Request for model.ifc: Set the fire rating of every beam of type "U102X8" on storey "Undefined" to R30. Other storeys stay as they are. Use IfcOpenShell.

First a look at what the model holds.

```python
import ifcopenshell
import ifcopenshell.util.element

model = ifcopenshell.open("model.ifc")
print(model.schema)
storey = next(s for s in model.by_type("IfcBuildingStorey") if s.Name == "Undefined")
beams = [e for e in ifcopenshell.util.element.get_decomposition(storey) if e.is_a("IfcBeam")]
seen = {}
for e in beams:
    element_type = ifcopenshell.util.element.get_type(e)
    key = (element_type.Name if element_type != e and element_type else None, ifcopenshell.util.element.get_pset(e, "Pset_BeamCommon", "FireRating"))
    seen[key] = seen.get(key, 0) + 1
for (name, value), count in sorted(seen.items(), key=str):
    print(count, "x", name, "|", value)
```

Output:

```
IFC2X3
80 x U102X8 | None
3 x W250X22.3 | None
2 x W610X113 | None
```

```python
import ifcopenshell
import ifcopenshell.api.pset
import ifcopenshell.util.element

model = ifcopenshell.open("model.ifc")

storey = next(s for s in model.by_type("IfcBuildingStorey") if s.Name == "Undefined")
beams = [e for e in ifcopenshell.util.element.get_decomposition(storey) if e.is_a("IfcBeam")]

count = 0
for e in beams:
    element_type = ifcopenshell.util.element.get_type(e)
    if element_type in (None, e) or element_type.Name != "U102X8":
        continue
    found = ifcopenshell.util.element.get_pset(e, "Pset_BeamCommon", should_inherit=False)
    if found:
        pset = model.by_id(found["id"])
        if len(ifcopenshell.util.element.get_elements_by_pset(pset)) > 1:
            pset = ifcopenshell.api.pset.unshare_pset(model, products=[e], pset=pset)[0]
    else:
        pset = ifcopenshell.api.pset.add_pset(model, product=e, name="Pset_BeamCommon")
    ifcopenshell.api.pset.edit_pset(model, pset=pset, properties={"FireRating": "R30"})
    count += 1

print(count, "beams updated")

model.write("model_edited.ifc")
```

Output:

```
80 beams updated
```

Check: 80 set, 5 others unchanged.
